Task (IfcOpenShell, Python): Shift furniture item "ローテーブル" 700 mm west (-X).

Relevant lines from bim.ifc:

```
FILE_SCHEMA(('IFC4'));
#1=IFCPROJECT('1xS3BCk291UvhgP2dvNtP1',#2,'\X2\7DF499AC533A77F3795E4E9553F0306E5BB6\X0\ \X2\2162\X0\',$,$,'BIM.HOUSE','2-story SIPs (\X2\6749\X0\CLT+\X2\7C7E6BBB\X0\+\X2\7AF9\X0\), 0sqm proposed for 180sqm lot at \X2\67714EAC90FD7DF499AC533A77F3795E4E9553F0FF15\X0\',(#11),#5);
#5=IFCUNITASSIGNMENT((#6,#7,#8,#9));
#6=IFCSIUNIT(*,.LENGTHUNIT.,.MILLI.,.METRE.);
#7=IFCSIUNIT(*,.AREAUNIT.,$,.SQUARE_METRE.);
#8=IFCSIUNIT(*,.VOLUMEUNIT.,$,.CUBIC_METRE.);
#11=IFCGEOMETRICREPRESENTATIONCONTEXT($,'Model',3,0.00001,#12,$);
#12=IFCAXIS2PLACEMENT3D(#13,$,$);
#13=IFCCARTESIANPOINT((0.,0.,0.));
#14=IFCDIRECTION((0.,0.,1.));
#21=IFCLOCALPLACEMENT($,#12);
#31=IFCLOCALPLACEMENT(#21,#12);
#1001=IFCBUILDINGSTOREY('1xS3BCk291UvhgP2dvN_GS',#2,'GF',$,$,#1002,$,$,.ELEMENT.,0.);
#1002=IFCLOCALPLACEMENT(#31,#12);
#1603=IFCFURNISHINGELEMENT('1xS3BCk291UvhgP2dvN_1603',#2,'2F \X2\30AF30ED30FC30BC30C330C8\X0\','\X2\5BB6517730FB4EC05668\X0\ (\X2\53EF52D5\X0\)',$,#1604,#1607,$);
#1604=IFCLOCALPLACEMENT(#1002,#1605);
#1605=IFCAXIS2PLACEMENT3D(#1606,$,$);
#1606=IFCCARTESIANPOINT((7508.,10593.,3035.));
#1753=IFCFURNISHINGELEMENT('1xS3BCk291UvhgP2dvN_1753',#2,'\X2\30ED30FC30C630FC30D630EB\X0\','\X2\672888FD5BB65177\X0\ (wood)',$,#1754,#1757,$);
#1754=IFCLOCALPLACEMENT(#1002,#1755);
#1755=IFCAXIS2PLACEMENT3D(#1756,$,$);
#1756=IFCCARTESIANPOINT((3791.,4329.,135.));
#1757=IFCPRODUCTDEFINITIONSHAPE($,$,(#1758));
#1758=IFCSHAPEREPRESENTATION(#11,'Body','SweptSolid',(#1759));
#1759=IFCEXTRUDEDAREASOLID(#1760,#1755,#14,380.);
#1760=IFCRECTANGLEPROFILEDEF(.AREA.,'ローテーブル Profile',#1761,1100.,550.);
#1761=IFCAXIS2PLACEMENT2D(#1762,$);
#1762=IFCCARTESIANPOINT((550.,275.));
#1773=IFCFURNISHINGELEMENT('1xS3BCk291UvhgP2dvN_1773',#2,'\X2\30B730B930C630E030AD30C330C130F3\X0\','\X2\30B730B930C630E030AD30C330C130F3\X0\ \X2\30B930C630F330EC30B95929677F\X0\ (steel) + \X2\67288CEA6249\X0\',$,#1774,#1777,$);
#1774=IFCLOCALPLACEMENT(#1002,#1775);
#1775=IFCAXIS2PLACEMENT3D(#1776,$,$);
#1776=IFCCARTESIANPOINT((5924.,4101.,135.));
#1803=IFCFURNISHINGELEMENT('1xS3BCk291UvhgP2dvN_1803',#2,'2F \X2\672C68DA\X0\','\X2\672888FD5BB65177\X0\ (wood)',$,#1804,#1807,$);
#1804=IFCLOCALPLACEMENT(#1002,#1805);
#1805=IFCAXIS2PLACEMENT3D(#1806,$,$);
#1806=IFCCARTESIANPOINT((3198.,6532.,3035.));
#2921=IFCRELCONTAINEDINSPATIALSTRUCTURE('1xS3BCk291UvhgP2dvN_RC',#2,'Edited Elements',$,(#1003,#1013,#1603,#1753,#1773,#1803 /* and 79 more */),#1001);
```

```python
import ifcopenshell
import ifcopenshell.api.geometry
import ifcopenshell.util.placement
import ifcopenshell.util.unit

model = ifcopenshell.open("bim.ifc")
unit_scale = ifcopenshell.util.unit.calculate_unit_scale(model)

item = model.by_guid("1xS3BCk291UvhgP2dvN_1753")
matrix = ifcopenshell.util.placement.get_local_placement(item.ObjectPlacement)
matrix[0, 3] -= 0.7 / unit_scale
ifcopenshell.api.geometry.edit_object_placement(model, product=item, matrix=matrix, is_si=False)

print(ifcopenshell.util.placement.get_local_placement(item.ObjectPlacement).round(3) + 0.0)

model.write("bim_v2.ifc")
```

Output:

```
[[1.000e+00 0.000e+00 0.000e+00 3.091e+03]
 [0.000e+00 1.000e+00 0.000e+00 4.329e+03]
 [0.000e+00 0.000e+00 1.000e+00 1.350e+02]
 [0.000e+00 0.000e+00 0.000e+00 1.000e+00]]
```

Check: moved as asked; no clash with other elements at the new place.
